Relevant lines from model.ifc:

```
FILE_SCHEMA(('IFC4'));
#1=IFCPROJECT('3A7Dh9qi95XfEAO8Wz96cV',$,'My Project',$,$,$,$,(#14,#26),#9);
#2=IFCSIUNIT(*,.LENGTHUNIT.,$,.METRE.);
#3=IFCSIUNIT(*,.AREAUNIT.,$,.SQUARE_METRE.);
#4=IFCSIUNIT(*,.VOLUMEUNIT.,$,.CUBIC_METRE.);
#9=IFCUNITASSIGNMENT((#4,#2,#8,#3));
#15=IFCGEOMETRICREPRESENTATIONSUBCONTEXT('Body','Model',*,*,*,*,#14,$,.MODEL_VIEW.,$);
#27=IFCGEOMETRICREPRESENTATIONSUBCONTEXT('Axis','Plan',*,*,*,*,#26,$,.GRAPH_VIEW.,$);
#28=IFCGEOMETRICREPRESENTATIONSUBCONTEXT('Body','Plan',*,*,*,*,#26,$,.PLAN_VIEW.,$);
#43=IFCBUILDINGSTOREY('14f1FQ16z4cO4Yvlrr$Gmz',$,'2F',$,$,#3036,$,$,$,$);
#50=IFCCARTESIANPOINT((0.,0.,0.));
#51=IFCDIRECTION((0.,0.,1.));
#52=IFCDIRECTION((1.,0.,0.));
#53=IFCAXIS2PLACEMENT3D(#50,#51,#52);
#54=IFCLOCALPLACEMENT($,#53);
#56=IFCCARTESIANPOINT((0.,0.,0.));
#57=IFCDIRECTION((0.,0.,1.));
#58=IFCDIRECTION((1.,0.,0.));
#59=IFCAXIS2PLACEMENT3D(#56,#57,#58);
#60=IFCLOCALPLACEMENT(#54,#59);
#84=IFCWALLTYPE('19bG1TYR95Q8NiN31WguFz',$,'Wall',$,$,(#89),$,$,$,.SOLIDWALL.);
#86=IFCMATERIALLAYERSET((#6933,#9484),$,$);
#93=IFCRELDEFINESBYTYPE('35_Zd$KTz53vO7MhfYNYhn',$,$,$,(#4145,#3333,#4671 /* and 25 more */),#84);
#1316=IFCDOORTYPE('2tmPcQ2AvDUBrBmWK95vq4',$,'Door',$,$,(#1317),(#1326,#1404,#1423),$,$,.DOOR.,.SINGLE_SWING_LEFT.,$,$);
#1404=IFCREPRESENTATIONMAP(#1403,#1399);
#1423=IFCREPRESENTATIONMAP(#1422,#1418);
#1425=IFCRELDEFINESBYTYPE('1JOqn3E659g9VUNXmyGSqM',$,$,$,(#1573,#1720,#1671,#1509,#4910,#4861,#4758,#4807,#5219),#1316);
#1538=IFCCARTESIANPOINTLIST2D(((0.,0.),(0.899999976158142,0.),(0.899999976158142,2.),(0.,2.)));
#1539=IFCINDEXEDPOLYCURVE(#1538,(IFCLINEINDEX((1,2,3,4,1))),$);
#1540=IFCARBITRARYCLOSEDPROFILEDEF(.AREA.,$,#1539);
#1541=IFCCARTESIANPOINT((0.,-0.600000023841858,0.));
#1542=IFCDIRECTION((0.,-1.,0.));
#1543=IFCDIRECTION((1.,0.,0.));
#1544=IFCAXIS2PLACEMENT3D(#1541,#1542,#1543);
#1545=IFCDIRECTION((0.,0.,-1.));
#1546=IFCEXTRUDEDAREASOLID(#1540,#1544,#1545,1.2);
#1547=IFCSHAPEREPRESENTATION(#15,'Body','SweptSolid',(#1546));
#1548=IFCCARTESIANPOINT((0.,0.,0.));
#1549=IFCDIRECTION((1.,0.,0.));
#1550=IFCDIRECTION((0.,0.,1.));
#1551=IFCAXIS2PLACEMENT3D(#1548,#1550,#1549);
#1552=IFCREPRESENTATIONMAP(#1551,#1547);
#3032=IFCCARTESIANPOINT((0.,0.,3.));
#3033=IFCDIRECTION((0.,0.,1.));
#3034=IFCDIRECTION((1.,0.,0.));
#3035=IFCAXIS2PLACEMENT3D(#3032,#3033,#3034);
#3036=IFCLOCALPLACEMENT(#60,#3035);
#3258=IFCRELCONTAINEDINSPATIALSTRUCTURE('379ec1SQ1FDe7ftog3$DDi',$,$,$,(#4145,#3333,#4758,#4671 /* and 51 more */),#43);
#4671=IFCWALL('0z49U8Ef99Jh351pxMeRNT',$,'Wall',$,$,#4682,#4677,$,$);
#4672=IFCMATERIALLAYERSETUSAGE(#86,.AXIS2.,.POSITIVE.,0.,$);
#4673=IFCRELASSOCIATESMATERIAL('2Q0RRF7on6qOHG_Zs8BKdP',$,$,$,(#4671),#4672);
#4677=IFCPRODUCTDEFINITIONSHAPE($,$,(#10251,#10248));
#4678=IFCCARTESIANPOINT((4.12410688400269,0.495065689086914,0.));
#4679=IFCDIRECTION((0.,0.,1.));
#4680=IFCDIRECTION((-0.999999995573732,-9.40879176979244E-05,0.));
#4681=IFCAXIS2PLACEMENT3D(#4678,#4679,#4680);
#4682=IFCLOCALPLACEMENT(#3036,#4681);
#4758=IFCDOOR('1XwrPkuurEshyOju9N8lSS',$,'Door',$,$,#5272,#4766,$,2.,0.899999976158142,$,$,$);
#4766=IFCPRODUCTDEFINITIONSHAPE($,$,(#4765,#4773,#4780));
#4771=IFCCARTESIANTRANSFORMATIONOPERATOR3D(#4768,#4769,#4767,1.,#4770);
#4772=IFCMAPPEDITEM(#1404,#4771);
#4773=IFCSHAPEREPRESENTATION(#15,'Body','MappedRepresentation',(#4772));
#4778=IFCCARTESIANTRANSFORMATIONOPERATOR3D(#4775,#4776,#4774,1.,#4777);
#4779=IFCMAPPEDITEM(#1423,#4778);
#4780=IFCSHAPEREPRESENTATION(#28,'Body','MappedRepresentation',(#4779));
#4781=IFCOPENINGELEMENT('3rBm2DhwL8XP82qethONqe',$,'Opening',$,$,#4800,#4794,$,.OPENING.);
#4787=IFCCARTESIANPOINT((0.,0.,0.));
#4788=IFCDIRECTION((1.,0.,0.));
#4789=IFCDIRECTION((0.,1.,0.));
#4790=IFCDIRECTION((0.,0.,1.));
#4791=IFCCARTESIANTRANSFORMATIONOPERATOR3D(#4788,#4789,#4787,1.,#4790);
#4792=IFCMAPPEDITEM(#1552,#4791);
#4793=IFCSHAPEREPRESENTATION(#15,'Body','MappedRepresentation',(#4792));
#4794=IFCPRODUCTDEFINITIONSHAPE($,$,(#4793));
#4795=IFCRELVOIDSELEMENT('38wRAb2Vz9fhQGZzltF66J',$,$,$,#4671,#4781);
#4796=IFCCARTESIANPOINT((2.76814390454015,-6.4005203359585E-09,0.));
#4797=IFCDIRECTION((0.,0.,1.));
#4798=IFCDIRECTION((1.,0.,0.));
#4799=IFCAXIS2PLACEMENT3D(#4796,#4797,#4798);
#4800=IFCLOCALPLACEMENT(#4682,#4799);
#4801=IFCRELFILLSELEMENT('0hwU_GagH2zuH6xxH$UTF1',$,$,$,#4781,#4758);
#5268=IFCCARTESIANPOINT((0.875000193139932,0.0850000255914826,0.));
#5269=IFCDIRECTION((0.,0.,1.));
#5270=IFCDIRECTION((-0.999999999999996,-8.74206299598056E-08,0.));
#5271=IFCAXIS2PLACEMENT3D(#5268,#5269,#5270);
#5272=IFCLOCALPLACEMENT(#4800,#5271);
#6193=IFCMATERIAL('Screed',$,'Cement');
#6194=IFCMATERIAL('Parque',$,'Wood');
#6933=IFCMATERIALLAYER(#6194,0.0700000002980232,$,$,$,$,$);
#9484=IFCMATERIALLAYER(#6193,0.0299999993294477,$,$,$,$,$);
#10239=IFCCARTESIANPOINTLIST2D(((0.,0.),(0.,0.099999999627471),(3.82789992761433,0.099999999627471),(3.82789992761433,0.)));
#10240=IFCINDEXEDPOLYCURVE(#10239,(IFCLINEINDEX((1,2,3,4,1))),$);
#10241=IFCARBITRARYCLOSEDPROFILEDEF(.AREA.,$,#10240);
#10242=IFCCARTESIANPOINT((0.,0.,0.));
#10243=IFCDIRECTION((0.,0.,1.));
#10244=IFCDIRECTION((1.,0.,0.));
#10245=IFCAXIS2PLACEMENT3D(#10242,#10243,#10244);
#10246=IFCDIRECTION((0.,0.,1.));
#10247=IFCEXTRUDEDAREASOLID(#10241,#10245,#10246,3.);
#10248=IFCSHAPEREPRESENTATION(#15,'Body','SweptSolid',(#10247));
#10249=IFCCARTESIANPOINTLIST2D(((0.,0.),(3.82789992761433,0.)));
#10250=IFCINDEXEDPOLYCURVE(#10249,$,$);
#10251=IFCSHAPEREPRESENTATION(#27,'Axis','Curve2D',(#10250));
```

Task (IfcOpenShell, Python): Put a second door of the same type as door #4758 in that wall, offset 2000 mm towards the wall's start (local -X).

```python
import ifcopenshell
import ifcopenshell.api.feature
import ifcopenshell.api.geometry
import ifcopenshell.api.root
import ifcopenshell.geom
import ifcopenshell.util.element
import ifcopenshell.util.placement
import ifcopenshell.util.shape
import ifcopenshell.util.unit

model = ifcopenshell.open("model.ifc")
unit_scale = ifcopenshell.util.unit.calculate_unit_scale(model)
settings = ifcopenshell.geom.settings()


def volume(element):
    """Net volume in cubic metres, openings subtracted."""
    shape = ifcopenshell.geom.create_shape(settings, element)
    return ifcopenshell.util.shape.get_volume(shape.geometry)


door = model.by_id(4758)
opening = door.FillsVoids[0].RelatingOpeningElement
wall = opening.VoidsElements[0].RelatingBuildingElement
before = volume(wall)
shift = ifcopenshell.util.placement.get_local_placement(wall.ObjectPlacement)[:3, 0] * -2 / unit_scale

# copy_class copies the void relationship, type, container and properties, but no geometry.
new_opening = ifcopenshell.api.root.copy_class(model, product=opening)
new_opening.Representation = ifcopenshell.util.element.copy_deep(
    model, opening.Representation, exclude=["IfcGeometricRepresentationContext", "IfcRepresentationMap"]
)
new_door = ifcopenshell.api.root.copy_class(model, product=door)
new_door.Representation = ifcopenshell.util.element.copy_deep(
    model, door.Representation, exclude=["IfcGeometricRepresentationContext", "IfcRepresentationMap"]
)
ifcopenshell.api.feature.add_filling(model, opening=new_opening, element=new_door)

for old, new in ((opening, new_opening), (door, new_door)):
    matrix = ifcopenshell.util.placement.get_local_placement(old.ObjectPlacement)
    matrix[:3, 3] += shift
    ifcopenshell.api.geometry.edit_object_placement(model, product=new, matrix=matrix, is_si=False)

after = volume(wall)

print(f"wall volume {before:.3f} -> {after:.3f} m3")

model.write("model-out.ifc")
```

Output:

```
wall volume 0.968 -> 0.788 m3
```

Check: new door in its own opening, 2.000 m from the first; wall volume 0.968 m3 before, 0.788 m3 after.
